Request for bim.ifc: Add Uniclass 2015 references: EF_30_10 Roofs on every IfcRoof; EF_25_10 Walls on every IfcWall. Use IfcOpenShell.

First a look at what the model holds.

```python
import ifcopenshell

model = ifcopenshell.open("bim.ifc")
print(model.schema)
print("classifications:", [c.Name for c in model.by_type("IfcClassification")])
for ifc_class in ("IfcDoor", "IfcRoof", "IfcStair", "IfcWall", "IfcWindow"):
    print(ifc_class, len(model.by_type(ifc_class)))
```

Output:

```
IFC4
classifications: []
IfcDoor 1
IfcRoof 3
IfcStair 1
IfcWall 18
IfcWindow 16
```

```python
import ifcopenshell
import ifcopenshell.api.classification

model = ifcopenshell.open("bim.ifc")

system = ifcopenshell.api.classification.add_classification(model, classification="Uniclass 2015")

codes = {
    "IfcRoof": ("EF_30_10", "Roofs"),
    "IfcWall": ("EF_25_10", "Walls"),
}
for ifc_class, (code, name) in codes.items():
    products = model.by_type(ifc_class)
    ifcopenshell.api.classification.add_reference(
        model, products=products, classification=system, identification=code, name=name
    )
    print(code, len(products))

model.write("bim_updated.ifc")
```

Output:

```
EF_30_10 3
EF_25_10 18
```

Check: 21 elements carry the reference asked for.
